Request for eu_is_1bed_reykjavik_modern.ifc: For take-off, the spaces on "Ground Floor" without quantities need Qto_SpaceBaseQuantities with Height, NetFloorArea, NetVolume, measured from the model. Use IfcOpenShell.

First a look at what the model holds.

```python
import ifcopenshell
import ifcopenshell.util.element
import ifcopenshell.util.unit

model = ifcopenshell.open("eu_is_1bed_reykjavik_modern.ifc")
print(model.schema)
for unit_type in ("LENGTHUNIT", "AREAUNIT", "VOLUMEUNIT"):
    print(unit_type, ifcopenshell.util.unit.calculate_unit_scale(model, unit_type))
storey = next(s for s in model.by_type("IfcBuildingStorey") if s.Name == "Ground Floor")
spaces = [e for e in ifcopenshell.util.element.get_decomposition(storey) if e.is_a("IfcSpace")]
for e in sorted(spaces, key=lambda e: e.id()):
    print(e.id(), e.is_a(), e.Name, list(ifcopenshell.util.element.get_psets(e, qtos_only=True)), sep=" | ")
```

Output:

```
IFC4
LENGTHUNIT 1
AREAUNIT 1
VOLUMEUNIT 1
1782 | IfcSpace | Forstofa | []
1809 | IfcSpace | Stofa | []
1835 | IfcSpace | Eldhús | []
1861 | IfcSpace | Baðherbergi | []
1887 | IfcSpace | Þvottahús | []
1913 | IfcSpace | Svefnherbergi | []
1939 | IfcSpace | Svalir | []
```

```python
import ifcopenshell
import ifcopenshell.api.pset
import ifcopenshell.geom
import ifcopenshell.util.element
import ifcopenshell.util.shape
import ifcopenshell.util.unit

model = ifcopenshell.open("eu_is_1bed_reykjavik_modern.ifc")
unit_scale = ifcopenshell.util.unit.calculate_unit_scale(model)
area_scale = ifcopenshell.util.unit.calculate_unit_scale(model, "AREAUNIT")
volume_scale = ifcopenshell.util.unit.calculate_unit_scale(model, "VOLUMEUNIT")
settings = ifcopenshell.geom.settings()

storey = next(s for s in model.by_type("IfcBuildingStorey") if s.Name == "Ground Floor")
spaces = [e for e in ifcopenshell.util.element.get_decomposition(storey) if e.is_a("IfcSpace")]

for e in sorted(spaces, key=lambda e: e.id()):
    if ifcopenshell.util.element.get_psets(e, qtos_only=True, should_inherit=False):
        continue
    # Geometry comes back in metres, in the element's own axes.
    shape = ifcopenshell.geom.create_shape(settings, e)
    values = {
        "Height": ifcopenshell.util.shape.get_z(shape.geometry) / unit_scale,
        "NetFloorArea": ifcopenshell.util.shape.get_footprint_area(shape.geometry) / area_scale,
        "NetVolume": ifcopenshell.util.shape.get_volume(shape.geometry) / volume_scale,
    }
    qto = ifcopenshell.api.pset.add_qto(model, product=e, name="Qto_SpaceBaseQuantities")
    ifcopenshell.api.pset.edit_qto(model, qto=qto, properties=values)
    print(e.id(), {k: round(v, 3) for k, v in values.items()})

model.write("eu_is_1bed_reykjavik_modern_updated.ifc")
```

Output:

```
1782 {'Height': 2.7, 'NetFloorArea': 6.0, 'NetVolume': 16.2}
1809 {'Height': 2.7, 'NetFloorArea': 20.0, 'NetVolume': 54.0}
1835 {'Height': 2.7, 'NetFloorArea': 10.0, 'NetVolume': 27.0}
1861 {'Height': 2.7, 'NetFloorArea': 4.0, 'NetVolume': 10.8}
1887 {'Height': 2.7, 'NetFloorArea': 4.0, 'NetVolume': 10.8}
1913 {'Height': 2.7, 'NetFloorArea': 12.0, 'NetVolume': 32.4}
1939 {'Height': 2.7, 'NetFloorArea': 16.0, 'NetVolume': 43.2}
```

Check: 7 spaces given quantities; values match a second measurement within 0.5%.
